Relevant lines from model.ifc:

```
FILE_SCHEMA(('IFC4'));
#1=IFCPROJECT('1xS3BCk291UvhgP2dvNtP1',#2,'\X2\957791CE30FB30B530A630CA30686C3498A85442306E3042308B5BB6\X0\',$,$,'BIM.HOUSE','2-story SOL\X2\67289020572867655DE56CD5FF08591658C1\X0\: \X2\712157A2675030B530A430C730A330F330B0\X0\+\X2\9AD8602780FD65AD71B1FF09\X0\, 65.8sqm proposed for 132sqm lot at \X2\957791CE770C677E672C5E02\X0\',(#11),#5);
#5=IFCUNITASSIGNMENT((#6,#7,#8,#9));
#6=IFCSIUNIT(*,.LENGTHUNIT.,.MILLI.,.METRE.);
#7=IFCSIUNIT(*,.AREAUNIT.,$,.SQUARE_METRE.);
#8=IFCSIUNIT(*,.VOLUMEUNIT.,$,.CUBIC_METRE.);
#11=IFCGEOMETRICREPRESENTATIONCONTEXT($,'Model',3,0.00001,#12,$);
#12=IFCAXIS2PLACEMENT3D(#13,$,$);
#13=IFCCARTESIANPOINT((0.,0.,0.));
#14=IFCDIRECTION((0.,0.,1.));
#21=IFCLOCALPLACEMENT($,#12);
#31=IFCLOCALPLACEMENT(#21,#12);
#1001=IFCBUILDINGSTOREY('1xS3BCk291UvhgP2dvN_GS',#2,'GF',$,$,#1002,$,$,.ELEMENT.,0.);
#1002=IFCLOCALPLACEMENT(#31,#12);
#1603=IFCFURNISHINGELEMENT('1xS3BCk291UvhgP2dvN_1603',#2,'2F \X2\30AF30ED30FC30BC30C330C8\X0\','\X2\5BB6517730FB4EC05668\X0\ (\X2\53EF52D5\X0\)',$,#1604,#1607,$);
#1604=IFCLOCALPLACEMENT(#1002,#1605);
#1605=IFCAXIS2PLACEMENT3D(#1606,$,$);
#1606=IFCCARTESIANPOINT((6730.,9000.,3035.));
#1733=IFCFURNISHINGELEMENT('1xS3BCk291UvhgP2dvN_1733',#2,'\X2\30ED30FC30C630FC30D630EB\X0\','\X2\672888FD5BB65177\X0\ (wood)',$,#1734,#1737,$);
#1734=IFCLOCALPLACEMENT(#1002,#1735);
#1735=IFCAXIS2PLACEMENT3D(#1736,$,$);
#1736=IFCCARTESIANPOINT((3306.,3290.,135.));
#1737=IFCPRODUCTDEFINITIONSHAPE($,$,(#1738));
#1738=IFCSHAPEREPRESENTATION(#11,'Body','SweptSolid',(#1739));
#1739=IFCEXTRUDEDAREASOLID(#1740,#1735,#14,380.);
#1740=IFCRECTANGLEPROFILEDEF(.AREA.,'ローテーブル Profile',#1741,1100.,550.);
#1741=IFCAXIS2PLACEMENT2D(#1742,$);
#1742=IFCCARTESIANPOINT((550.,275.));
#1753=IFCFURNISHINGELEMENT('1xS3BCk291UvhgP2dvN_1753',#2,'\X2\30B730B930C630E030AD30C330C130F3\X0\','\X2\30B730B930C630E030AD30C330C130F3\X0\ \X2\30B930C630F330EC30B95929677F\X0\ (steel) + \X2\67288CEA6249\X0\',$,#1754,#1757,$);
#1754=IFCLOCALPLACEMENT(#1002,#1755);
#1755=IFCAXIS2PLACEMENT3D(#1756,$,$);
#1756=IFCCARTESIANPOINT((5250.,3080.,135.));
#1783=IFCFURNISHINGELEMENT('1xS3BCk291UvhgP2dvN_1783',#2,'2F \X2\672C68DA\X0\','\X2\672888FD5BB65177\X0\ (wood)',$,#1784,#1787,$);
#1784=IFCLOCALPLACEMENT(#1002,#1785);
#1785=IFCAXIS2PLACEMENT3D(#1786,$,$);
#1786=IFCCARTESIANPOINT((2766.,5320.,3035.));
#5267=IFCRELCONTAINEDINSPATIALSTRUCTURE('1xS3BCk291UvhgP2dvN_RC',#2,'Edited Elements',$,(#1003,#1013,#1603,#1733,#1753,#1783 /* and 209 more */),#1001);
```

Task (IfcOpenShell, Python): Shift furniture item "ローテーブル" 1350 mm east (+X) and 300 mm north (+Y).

```python
import ifcopenshell
import ifcopenshell.api.geometry
import ifcopenshell.util.placement
import ifcopenshell.util.unit

model = ifcopenshell.open("model.ifc")
unit_scale = ifcopenshell.util.unit.calculate_unit_scale(model)

item = model.by_guid("1xS3BCk291UvhgP2dvN_1733")
matrix = ifcopenshell.util.placement.get_local_placement(item.ObjectPlacement)
matrix[0, 3] += 1.35 / unit_scale
matrix[1, 3] += 0.3 / unit_scale
ifcopenshell.api.geometry.edit_object_placement(model, product=item, matrix=matrix, is_si=False)

print(ifcopenshell.util.placement.get_local_placement(item.ObjectPlacement).round(3) + 0.0)

model.write("model_rev.ifc")
```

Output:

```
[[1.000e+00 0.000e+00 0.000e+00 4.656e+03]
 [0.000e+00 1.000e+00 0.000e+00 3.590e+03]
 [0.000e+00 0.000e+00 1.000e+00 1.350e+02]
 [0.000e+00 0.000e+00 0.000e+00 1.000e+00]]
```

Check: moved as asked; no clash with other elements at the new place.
